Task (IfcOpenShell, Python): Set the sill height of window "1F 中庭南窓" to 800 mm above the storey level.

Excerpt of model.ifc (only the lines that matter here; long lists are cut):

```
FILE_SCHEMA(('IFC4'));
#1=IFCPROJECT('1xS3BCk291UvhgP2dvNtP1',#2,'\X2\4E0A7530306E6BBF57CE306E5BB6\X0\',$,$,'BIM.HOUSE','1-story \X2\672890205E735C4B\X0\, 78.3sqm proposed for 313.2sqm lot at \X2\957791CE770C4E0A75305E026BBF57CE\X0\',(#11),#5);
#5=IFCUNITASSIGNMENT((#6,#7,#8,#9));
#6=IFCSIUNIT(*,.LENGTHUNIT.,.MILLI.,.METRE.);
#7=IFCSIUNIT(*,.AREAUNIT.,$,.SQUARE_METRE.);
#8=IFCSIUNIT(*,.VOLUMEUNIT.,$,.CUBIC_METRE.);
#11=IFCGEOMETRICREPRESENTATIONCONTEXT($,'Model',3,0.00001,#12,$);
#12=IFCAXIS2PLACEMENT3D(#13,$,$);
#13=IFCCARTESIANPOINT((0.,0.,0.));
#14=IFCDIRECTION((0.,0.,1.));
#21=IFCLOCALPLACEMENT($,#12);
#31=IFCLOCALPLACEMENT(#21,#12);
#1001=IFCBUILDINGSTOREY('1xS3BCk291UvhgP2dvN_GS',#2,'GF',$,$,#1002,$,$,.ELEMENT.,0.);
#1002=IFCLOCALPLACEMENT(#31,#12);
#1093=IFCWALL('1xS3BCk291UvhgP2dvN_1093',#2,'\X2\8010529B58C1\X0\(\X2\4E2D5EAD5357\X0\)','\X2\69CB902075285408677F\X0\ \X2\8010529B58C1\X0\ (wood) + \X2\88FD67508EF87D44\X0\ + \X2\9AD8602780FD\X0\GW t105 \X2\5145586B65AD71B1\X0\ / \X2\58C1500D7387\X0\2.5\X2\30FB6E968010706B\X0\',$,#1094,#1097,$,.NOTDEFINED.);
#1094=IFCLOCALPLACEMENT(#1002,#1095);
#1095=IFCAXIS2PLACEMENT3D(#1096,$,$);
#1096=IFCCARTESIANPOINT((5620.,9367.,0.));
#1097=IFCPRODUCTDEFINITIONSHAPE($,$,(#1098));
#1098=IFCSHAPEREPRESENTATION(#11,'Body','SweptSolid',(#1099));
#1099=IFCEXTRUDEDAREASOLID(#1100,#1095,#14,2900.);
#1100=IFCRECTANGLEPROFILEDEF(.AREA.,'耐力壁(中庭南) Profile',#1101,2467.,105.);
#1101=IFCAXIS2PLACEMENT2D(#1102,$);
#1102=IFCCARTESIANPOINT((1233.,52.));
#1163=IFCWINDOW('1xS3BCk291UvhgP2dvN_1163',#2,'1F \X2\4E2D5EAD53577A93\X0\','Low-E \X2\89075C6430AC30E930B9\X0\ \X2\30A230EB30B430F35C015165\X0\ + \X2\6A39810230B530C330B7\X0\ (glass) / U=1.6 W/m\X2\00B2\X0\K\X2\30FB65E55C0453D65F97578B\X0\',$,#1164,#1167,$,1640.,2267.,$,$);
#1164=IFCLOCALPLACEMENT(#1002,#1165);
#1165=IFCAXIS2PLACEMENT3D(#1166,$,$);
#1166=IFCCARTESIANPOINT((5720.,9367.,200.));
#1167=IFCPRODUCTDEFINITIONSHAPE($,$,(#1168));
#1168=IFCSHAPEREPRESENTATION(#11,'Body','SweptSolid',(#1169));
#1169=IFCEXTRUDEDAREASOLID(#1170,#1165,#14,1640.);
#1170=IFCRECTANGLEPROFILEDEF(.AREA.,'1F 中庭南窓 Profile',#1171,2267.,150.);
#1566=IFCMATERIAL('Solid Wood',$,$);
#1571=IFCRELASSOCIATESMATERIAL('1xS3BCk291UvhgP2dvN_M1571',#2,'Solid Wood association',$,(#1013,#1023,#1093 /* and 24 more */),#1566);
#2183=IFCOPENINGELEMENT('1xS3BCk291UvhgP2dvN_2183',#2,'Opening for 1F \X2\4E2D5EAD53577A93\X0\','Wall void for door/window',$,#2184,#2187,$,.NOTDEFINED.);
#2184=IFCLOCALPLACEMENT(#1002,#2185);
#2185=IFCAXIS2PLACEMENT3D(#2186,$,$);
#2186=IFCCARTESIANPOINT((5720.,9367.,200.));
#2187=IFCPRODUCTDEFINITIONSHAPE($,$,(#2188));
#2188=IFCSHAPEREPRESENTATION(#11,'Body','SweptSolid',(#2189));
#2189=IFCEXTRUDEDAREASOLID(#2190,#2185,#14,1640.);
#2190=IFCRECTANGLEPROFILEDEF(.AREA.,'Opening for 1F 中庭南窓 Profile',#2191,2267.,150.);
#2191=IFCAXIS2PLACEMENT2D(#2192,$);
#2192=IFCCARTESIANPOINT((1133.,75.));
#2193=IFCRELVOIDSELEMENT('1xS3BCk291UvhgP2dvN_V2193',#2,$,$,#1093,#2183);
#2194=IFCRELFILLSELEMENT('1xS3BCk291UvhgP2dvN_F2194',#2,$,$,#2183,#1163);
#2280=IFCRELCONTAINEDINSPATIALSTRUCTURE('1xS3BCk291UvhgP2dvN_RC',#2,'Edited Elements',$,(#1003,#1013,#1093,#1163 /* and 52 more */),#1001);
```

```python
import numpy as np
import ifcopenshell
import ifcopenshell.api.geometry
import ifcopenshell.geom
import ifcopenshell.util.element
import ifcopenshell.util.placement
import ifcopenshell.util.shape
import ifcopenshell.util.unit

model = ifcopenshell.open("model.ifc")
unit_scale = ifcopenshell.util.unit.calculate_unit_scale(model)

window = model.by_guid("1xS3BCk291UvhgP2dvN_1163")
opening = window.FillsVoids[0].RelatingOpeningElement
storey = ifcopenshell.util.element.get_container(window, ifc_class="IfcBuildingStorey")
level = ifcopenshell.util.placement.get_local_placement(storey.ObjectPlacement)[2, 3]

# The opening's origin need not be at the sill, so measure its lowest point.
shape = ifcopenshell.geom.create_shape(ifcopenshell.geom.settings(), opening)
bottom = ifcopenshell.util.shape.get_shape_bottom_elevation(shape, shape.geometry) / unit_scale
dz = level + 800.0 - bottom

shift = np.array([0.0, 0.0, dz])
# The window is not placed relative to its opening, so move both.
for product in (opening, window):
    matrix = ifcopenshell.util.placement.get_local_placement(product.ObjectPlacement)
    matrix[:3, 3] += shift
    ifcopenshell.api.geometry.edit_object_placement(model, product=product, matrix=matrix, is_si=False)

print(f"moved by {dz * unit_scale:+.3f} m")

model.write("model_updated.ifc")
```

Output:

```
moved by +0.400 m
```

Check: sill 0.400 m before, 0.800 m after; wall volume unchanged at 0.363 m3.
